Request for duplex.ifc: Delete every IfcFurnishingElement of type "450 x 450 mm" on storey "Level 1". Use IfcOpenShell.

First a look at what the model holds.

```python
import ifcopenshell
import ifcopenshell.util.element

model = ifcopenshell.open("duplex.ifc")
print(model.schema)
storey = next(s for s in model.by_type("IfcBuildingStorey") if s.Name == "Level 1")
furniture = [e for e in ifcopenshell.util.element.get_decomposition(storey) if e.is_a("IfcFurnishingElement")]
seen = {}
for e in furniture:
    element_type = ifcopenshell.util.element.get_type(e)
    name = element_type.Name if element_type not in (None, e) else None
    seen[name] = seen.get(name, 0) + 1
for name, count in sorted(seen.items(), key=str):
    print(count, "x", name)
```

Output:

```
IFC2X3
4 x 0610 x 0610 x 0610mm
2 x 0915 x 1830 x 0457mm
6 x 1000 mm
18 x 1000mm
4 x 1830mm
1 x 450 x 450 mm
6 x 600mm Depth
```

```python
import ifcopenshell
import ifcopenshell.api.root
import ifcopenshell.util.element

model = ifcopenshell.open("duplex.ifc")

storey = next(s for s in model.by_type("IfcBuildingStorey") if s.Name == "Level 1")
furniture = [e for e in ifcopenshell.util.element.get_decomposition(storey) if e.is_a("IfcFurnishingElement")]
targets = [e for e in furniture if (t := ifcopenshell.util.element.get_type(e)) not in (None, e) and t.Name == "450 x 450 mm"]

for e in targets:
    ifcopenshell.api.root.remove_product(model, product=e)
print(len(targets), "removed")

model.write("duplex-out.ifc")
```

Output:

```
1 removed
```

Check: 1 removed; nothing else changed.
